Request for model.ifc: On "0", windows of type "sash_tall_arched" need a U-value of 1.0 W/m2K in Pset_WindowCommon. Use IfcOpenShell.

First a look at what the model holds.

```python
import ifcopenshell
import ifcopenshell.util.element

model = ifcopenshell.open("model.ifc")
print(model.schema)
storey = next(s for s in model.by_type("IfcBuildingStorey") if s.Name == "0")
windows = [e for e in ifcopenshell.util.element.get_decomposition(storey) if e.is_a("IfcWindow")]
seen = {}
for e in windows:
    element_type = ifcopenshell.util.element.get_type(e)
    key = (element_type.Name if element_type != e and element_type else None, ifcopenshell.util.element.get_pset(e, "Pset_WindowCommon", "ThermalTransmittance"))
    seen[key] = seen.get(key, 0) + 1
for (name, value), count in sorted(seen.items(), key=str):
    print(count, "x", name, "|", value)
```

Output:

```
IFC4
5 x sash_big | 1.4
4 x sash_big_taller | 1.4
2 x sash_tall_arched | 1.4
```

```python
import ifcopenshell
import ifcopenshell.api.pset
import ifcopenshell.util.element

model = ifcopenshell.open("model.ifc")

storey = next(s for s in model.by_type("IfcBuildingStorey") if s.Name == "0")
windows = [e for e in ifcopenshell.util.element.get_decomposition(storey) if e.is_a("IfcWindow")]

count = 0
for e in windows:
    element_type = ifcopenshell.util.element.get_type(e)
    if element_type in (None, e) or element_type.Name != "sash_tall_arched":
        continue
    # add_pset returns the element's existing set when there is one.
    pset = ifcopenshell.api.pset.add_pset(model, product=e, name="Pset_WindowCommon")
    ifcopenshell.api.pset.edit_pset(model, pset=pset, properties={"ThermalTransmittance": 1.0})
    count += 1

print(count, "windows updated")

model.write("model_updated.ifc")
```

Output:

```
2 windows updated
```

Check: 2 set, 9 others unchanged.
